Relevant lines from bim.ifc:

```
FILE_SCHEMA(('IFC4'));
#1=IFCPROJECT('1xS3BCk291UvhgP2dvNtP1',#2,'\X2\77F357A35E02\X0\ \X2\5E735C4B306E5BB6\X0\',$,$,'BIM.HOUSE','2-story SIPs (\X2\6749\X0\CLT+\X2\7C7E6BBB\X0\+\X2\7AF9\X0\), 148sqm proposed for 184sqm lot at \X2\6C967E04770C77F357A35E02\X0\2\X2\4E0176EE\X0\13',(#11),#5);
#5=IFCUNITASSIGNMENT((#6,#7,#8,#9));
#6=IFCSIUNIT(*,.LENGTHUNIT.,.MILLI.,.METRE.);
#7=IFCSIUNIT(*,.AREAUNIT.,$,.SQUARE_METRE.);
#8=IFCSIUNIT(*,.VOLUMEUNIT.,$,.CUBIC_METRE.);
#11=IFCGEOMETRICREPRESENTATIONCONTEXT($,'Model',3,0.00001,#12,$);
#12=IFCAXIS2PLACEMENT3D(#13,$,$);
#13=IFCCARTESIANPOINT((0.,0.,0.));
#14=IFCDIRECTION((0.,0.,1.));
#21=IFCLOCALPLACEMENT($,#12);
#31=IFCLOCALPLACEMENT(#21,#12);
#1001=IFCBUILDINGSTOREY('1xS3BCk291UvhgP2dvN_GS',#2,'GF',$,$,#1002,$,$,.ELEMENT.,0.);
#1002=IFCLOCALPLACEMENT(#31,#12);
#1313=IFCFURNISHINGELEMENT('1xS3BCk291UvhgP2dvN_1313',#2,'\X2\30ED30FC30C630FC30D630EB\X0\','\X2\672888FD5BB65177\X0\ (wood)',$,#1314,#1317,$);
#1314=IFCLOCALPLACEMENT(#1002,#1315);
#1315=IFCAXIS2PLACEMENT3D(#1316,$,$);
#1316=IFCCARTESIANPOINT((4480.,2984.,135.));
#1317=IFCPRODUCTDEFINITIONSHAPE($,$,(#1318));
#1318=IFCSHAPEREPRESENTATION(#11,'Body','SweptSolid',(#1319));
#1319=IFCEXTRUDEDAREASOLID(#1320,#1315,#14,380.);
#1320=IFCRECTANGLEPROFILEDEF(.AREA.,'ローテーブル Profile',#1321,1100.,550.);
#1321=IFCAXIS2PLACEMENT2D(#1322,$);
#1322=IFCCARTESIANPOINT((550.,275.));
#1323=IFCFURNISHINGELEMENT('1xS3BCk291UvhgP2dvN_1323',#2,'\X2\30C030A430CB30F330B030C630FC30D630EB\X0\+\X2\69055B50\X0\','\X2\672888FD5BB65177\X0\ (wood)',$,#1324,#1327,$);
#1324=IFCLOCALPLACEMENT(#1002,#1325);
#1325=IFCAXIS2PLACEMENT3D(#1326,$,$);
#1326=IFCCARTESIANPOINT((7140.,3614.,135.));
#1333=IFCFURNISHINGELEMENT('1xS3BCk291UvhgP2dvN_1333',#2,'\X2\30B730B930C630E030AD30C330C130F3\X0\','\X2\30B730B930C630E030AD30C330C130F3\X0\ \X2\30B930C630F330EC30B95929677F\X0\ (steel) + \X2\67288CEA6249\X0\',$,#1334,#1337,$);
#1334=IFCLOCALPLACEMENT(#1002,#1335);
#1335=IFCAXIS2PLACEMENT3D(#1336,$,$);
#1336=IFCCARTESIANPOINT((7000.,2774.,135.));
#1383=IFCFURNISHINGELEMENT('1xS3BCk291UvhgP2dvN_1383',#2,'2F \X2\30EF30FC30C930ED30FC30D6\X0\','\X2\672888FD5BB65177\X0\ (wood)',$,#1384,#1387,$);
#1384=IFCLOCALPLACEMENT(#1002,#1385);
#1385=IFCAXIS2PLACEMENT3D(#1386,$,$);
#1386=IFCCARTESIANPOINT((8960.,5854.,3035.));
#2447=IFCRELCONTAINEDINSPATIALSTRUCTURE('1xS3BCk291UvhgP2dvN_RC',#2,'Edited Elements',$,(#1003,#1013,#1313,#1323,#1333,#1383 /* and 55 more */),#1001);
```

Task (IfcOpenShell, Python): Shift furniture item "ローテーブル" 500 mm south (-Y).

```python
import ifcopenshell
import ifcopenshell.api.geometry
import ifcopenshell.util.placement
import ifcopenshell.util.unit

model = ifcopenshell.open("bim.ifc")
unit_scale = ifcopenshell.util.unit.calculate_unit_scale(model)

item = model.by_id(1313)
matrix = ifcopenshell.util.placement.get_local_placement(item.ObjectPlacement)
matrix[1, 3] -= 0.5 / unit_scale
ifcopenshell.api.geometry.edit_object_placement(model, product=item, matrix=matrix, is_si=False)

print(ifcopenshell.util.placement.get_local_placement(item.ObjectPlacement).round(3) + 0.0)

model.write("bim_rev.ifc")
```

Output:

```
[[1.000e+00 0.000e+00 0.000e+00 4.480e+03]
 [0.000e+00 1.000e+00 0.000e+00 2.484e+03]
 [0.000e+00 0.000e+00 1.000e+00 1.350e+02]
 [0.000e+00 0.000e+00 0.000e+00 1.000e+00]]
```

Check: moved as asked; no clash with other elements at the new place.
